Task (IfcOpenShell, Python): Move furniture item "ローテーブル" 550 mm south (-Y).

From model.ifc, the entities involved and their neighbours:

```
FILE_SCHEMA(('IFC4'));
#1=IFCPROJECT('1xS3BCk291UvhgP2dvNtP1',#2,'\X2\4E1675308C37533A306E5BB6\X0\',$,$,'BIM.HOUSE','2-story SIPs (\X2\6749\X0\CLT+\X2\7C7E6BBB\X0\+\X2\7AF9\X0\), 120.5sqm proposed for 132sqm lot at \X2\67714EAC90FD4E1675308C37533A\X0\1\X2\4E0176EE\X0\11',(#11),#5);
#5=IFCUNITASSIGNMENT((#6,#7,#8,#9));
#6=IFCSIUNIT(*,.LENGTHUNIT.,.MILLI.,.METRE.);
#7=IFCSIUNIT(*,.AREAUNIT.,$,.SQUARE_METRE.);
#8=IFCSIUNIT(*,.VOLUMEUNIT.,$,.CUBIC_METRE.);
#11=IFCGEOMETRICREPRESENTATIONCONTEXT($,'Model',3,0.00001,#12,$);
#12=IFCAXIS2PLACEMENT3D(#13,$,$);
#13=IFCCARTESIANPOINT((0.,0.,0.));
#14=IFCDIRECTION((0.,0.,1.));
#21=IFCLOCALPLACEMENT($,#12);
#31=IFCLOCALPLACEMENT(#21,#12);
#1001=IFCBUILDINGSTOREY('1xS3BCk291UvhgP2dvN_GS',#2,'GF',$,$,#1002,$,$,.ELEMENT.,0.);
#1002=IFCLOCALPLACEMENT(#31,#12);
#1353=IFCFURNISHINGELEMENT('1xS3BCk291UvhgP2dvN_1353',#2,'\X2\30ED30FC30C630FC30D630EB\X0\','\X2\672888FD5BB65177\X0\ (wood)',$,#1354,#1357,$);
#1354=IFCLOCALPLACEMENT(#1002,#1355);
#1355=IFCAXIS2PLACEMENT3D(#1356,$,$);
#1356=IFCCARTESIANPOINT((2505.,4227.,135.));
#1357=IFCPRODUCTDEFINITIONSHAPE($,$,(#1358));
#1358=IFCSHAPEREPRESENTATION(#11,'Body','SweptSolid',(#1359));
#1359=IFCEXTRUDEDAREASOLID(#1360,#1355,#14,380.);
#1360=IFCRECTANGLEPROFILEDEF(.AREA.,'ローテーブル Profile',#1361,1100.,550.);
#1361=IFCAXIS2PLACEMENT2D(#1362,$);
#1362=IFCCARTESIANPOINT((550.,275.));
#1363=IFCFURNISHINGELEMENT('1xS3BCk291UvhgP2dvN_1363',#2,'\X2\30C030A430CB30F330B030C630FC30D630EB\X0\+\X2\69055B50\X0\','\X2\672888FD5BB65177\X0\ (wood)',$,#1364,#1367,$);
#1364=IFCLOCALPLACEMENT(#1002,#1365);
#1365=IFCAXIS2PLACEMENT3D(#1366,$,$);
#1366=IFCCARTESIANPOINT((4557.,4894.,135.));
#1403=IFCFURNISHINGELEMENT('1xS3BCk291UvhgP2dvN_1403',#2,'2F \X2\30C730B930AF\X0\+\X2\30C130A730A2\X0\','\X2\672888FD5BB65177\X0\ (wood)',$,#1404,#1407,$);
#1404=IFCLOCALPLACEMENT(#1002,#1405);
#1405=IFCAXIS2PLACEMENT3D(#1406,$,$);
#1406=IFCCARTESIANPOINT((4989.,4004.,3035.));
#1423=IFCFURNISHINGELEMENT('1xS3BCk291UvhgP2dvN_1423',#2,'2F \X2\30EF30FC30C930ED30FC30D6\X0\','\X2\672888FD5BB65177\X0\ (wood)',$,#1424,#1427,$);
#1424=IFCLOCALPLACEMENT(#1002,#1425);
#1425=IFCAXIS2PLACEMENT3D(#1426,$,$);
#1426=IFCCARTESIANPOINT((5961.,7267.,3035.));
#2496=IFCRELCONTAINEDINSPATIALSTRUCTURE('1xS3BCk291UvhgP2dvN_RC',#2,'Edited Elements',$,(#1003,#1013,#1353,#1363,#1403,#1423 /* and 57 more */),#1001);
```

```python
import ifcopenshell
import ifcopenshell.api.geometry
import ifcopenshell.util.placement

model = ifcopenshell.open("model.ifc")

item = model.by_guid("1xS3BCk291UvhgP2dvN_1353")
matrix = ifcopenshell.util.placement.get_local_placement(item.ObjectPlacement)
matrix[1, 3] -= 550.0
ifcopenshell.api.geometry.edit_object_placement(model, product=item, matrix=matrix, is_si=False)

print(ifcopenshell.util.placement.get_local_placement(item.ObjectPlacement).round(3) + 0.0)

model.write("model-out.ifc")
```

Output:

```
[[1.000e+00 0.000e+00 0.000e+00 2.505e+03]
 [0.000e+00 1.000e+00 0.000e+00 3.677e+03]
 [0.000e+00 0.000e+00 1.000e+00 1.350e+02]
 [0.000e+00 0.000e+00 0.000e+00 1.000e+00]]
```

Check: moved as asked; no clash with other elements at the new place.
